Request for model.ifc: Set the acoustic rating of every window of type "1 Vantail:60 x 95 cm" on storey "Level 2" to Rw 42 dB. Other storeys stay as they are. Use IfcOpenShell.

First a look at what the model holds.

```python
import ifcopenshell
import ifcopenshell.util.element

model = ifcopenshell.open("model.ifc")
print(model.schema)
storey = next(s for s in model.by_type("IfcBuildingStorey") if s.Name == "Level 2")
windows = [e for e in ifcopenshell.util.element.get_decomposition(storey) if e.is_a("IfcWindow")]
seen = {}
for e in windows:
    element_type = ifcopenshell.util.element.get_type(e)
    key = (element_type.Name if element_type != e and element_type else None, ifcopenshell.util.element.get_pset(e, "Pset_WindowCommon", "AcousticRating"))
    seen[key] = seen.get(key, 0) + 1
for (name, value), count in sorted(seen.items(), key=str):
    print(count, "x", name, "|", value)
```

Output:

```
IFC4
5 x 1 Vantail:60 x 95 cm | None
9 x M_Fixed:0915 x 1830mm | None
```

```python
import ifcopenshell
import ifcopenshell.api.pset
import ifcopenshell.util.element

model = ifcopenshell.open("model.ifc")

storey = next(s for s in model.by_type("IfcBuildingStorey") if s.Name == "Level 2")
windows = [e for e in ifcopenshell.util.element.get_decomposition(storey) if e.is_a("IfcWindow")]

count = 0
for e in windows:
    element_type = ifcopenshell.util.element.get_type(e)
    if element_type in (None, e) or element_type.Name != "1 Vantail:60 x 95 cm":
        continue
    # add_pset returns the element's existing set when there is one.
    pset = ifcopenshell.api.pset.add_pset(model, product=e, name="Pset_WindowCommon")
    ifcopenshell.api.pset.edit_pset(model, pset=pset, properties={"AcousticRating": "Rw 42 dB"})
    count += 1

print(count, "windows updated")

model.write("model-out.ifc")
```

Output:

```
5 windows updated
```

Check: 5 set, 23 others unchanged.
